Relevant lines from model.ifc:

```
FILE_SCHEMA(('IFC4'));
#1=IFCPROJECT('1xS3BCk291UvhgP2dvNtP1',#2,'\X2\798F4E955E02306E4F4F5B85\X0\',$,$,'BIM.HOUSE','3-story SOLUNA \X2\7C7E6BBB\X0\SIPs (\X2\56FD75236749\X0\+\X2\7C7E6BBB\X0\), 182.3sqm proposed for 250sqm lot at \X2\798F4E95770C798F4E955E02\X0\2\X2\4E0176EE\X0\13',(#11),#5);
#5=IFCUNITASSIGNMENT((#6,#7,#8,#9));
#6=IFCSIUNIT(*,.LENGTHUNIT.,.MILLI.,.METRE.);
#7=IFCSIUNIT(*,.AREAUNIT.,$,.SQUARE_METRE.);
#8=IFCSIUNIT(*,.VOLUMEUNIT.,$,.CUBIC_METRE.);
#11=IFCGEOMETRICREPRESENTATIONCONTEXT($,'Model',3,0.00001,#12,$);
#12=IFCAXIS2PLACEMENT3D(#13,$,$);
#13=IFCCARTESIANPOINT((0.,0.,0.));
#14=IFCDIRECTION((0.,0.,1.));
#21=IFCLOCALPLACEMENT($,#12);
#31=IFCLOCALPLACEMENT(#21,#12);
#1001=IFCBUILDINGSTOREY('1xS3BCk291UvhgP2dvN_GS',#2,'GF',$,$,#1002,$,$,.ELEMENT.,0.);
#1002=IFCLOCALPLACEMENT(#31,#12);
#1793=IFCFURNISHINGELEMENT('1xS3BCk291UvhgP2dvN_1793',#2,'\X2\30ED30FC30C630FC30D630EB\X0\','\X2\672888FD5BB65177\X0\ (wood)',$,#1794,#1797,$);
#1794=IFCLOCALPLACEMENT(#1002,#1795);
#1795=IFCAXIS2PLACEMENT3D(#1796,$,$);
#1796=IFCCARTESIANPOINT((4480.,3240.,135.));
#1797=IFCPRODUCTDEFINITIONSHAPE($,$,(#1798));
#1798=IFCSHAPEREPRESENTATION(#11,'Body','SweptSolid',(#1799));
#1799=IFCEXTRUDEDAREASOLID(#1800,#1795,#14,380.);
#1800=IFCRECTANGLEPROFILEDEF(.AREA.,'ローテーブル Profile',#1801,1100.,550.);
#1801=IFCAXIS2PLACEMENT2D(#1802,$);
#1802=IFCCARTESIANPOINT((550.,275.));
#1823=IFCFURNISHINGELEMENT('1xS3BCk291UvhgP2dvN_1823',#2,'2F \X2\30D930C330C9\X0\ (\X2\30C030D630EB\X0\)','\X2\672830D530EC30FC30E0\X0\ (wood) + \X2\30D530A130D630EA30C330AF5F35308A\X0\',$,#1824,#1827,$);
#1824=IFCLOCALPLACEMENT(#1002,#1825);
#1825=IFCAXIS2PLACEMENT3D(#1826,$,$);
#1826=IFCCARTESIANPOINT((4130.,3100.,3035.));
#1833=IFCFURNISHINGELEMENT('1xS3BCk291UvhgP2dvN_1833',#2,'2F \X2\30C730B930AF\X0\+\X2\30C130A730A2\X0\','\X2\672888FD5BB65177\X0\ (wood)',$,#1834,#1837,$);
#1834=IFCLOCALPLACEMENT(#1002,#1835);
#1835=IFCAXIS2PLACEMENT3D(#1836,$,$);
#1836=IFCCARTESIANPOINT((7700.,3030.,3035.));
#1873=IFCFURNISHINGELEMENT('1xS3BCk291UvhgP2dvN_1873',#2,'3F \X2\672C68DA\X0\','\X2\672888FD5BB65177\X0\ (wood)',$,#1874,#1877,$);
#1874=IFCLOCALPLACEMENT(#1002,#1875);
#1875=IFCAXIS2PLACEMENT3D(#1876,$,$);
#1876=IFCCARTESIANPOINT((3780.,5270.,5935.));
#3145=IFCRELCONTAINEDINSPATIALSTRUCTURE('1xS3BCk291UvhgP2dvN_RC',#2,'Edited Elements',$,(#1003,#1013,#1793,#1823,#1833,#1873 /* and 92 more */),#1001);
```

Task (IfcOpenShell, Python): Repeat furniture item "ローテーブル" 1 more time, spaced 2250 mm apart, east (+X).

```python
import numpy as np
import ifcopenshell
import ifcopenshell.api.geometry
import ifcopenshell.api.root
import ifcopenshell.util.element
import ifcopenshell.util.placement
import ifcopenshell.util.unit

model = ifcopenshell.open("model.ifc")
unit_scale = ifcopenshell.util.unit.calculate_unit_scale(model)


def reuse_history(source, copy):
    """copy_class also copies each property set's owner history, people and application; keep the originals."""
    for rel in copy.IsDefinedBy:
        if rel.is_a("IfcRelDefinesByProperties") and (history := rel.RelatingPropertyDefinition.OwnerHistory):
            rel.RelatingPropertyDefinition.OwnerHistory = source.OwnerHistory
            ifcopenshell.util.element.remove_deep2(model, history)


source = model.by_guid("1xS3BCk291UvhgP2dvN_1793")
base = ifcopenshell.util.placement.get_local_placement(source.ObjectPlacement)
step = np.array([1.0, 0.0, 0.0]) * 2.25 / unit_scale

for i in range(1, 2):
    copy = ifcopenshell.api.root.copy_class(model, product=source)
    copy.Representation = ifcopenshell.util.element.copy_deep(
        model, source.Representation, exclude=["IfcGeometricRepresentationContext", "IfcRepresentationMap"]
    )
    reuse_history(source, copy)
    matrix = base.copy()
    matrix[:3, 3] += i * step
    print("added at", matrix[:3, 3].round(3) + 0.0)
    ifcopenshell.api.geometry.edit_object_placement(model, product=copy, matrix=matrix, is_si=False)

model.write("model_v2.ifc")
```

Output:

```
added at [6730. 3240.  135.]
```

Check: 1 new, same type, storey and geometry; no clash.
